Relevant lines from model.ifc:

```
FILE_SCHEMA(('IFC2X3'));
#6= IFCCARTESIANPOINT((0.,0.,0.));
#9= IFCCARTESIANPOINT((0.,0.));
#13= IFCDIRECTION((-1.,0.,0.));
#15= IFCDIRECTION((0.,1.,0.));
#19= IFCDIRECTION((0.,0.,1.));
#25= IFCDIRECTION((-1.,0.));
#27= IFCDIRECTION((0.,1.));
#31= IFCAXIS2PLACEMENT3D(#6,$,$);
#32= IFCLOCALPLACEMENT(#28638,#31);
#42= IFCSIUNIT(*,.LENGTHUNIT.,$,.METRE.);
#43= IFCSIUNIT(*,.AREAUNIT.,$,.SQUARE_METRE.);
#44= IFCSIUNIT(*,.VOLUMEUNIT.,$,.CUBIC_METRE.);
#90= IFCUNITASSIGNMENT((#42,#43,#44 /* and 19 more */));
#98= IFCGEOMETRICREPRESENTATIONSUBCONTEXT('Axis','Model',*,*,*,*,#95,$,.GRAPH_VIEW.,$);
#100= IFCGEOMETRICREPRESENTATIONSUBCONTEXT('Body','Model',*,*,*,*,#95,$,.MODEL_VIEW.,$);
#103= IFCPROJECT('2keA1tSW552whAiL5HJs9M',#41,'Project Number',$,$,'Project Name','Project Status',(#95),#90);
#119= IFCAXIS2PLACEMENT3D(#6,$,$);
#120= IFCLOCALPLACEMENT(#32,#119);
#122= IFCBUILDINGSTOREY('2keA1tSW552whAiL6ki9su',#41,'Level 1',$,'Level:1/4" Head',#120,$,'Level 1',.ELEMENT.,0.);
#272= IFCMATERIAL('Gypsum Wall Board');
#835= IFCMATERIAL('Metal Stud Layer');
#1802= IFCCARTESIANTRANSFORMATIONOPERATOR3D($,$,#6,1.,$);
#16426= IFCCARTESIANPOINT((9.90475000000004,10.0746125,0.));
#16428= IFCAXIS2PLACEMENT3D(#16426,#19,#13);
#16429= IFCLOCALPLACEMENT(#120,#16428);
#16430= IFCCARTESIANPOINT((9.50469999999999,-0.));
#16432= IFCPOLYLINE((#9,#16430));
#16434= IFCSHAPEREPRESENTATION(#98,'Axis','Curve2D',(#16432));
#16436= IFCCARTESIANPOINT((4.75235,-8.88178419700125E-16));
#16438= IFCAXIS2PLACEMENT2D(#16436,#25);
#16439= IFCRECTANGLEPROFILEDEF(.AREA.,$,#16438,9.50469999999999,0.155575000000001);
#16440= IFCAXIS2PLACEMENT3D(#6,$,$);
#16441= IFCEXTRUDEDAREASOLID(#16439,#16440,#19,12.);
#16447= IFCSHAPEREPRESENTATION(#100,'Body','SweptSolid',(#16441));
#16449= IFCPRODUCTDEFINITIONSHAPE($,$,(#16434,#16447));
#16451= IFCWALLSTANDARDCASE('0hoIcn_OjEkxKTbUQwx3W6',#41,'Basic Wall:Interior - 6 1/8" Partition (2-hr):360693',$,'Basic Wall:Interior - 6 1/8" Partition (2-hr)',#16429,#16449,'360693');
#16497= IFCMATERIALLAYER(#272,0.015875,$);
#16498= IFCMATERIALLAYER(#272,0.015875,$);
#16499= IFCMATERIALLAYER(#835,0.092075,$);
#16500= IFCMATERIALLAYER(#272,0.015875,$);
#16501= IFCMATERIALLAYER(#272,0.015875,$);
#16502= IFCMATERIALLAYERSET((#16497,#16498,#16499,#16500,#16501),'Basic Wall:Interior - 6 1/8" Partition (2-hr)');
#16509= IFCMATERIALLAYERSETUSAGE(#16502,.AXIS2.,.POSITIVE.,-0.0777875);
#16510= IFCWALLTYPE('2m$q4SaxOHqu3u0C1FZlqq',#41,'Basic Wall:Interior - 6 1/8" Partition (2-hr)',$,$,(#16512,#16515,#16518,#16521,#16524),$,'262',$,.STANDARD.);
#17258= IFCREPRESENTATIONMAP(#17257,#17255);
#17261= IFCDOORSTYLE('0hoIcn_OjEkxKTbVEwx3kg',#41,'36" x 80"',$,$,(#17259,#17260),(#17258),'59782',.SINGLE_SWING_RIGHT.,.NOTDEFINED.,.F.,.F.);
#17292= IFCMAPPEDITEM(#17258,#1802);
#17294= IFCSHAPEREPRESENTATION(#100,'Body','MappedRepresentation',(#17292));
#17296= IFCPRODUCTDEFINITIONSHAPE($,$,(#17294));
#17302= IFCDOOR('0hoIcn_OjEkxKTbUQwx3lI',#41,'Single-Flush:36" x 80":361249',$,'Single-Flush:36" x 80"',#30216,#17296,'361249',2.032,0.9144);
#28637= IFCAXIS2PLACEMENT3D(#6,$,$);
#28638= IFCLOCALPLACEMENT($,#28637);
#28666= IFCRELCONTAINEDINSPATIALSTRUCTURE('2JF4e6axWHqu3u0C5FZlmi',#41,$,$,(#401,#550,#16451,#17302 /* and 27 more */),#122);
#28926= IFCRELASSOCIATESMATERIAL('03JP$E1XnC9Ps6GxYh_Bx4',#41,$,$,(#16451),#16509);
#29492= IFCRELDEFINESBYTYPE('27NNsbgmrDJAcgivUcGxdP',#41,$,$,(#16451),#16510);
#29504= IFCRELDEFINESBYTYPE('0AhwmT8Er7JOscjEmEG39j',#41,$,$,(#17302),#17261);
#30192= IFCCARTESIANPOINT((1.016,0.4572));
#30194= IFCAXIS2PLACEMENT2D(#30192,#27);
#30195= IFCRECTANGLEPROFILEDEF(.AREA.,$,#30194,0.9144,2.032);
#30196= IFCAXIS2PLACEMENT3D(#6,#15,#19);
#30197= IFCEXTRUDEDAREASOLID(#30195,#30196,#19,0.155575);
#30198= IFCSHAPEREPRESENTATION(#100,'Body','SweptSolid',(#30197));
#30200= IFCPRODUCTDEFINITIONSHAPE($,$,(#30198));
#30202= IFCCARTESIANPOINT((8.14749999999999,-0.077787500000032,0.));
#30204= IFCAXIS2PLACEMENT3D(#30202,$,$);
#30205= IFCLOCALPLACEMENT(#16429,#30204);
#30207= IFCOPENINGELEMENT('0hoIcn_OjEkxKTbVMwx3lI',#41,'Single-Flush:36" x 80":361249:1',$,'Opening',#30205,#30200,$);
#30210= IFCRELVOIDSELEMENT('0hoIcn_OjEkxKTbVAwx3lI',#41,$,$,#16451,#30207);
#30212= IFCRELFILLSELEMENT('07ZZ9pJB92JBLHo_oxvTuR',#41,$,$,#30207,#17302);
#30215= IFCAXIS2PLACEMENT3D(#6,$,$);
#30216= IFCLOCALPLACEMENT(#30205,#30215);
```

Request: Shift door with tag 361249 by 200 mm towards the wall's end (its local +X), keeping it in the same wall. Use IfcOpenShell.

```python
import ifcopenshell
import ifcopenshell.api.geometry
import ifcopenshell.util.placement

model = ifcopenshell.open("model.ifc")

door = model.by_guid("0hoIcn_OjEkxKTbUQwx3lI")
opening = door.FillsVoids[0].RelatingOpeningElement
wall = opening.VoidsElements[0].RelatingBuildingElement

wall_matrix = ifcopenshell.util.placement.get_local_placement(wall.ObjectPlacement)
shift = wall_matrix[:3, 0] * 0.2
before = ifcopenshell.util.placement.get_local_placement(door.ObjectPlacement)[:3, 3].copy()

# The door is placed relative to its opening, so it follows when the opening moves.
matrix = ifcopenshell.util.placement.get_local_placement(opening.ObjectPlacement)
matrix[:3, 3] += shift
ifcopenshell.api.geometry.edit_object_placement(
    model, product=opening, matrix=matrix, is_si=False, should_transform_children=True
)

after = ifcopenshell.util.placement.get_local_placement(door.ObjectPlacement)[:3, 3]
print("door moved by", (after - before).round(3) + 0.0)

model.write("model_edited.ifc")
```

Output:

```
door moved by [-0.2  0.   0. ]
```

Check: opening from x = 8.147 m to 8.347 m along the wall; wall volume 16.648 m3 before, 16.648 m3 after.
